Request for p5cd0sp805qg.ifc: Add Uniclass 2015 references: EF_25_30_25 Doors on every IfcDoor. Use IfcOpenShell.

First a look at what the model holds.

```python
import ifcopenshell

model = ifcopenshell.open("p5cd0sp805qg.ifc")
print(model.schema)
print("classifications:", [c.Name for c in model.by_type("IfcClassification")])
for ifc_class in ("IfcDoor", "IfcRoof", "IfcStair", "IfcWall", "IfcWindow"):
    print(ifc_class, len(model.by_type(ifc_class)))
```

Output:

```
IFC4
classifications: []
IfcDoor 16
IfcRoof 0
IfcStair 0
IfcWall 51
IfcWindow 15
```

```python
import ifcopenshell
import ifcopenshell.api.classification

model = ifcopenshell.open("p5cd0sp805qg.ifc")

system = ifcopenshell.api.classification.add_classification(model, classification="Uniclass 2015")

codes = {
    "IfcDoor": ("EF_25_30_25", "Doors"),
}
for ifc_class, (code, name) in codes.items():
    products = model.by_type(ifc_class)
    ifcopenshell.api.classification.add_reference(
        model, products=products, classification=system, identification=code, name=name
    )
    print(code, len(products))

model.write("p5cd0sp805qg-out.ifc")
```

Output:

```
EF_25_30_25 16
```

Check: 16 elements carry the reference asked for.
